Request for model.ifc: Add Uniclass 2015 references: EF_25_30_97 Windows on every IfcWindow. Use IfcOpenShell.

First a look at what the model holds.

```python
import ifcopenshell

model = ifcopenshell.open("model.ifc")
print(model.schema)
print("classifications:", [c.Name for c in model.by_type("IfcClassification")])
for ifc_class in ("IfcDoor", "IfcRoof", "IfcStair", "IfcWall", "IfcWindow"):
    print(ifc_class, len(model.by_type(ifc_class)))
```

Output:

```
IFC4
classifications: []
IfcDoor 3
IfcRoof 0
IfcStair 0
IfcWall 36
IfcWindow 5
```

```python
import ifcopenshell
import ifcopenshell.api.classification

model = ifcopenshell.open("model.ifc")

system = ifcopenshell.api.classification.add_classification(model, classification="Uniclass 2015")

codes = {
    "IfcWindow": ("EF_25_30_97", "Windows"),
}
for ifc_class, (code, name) in codes.items():
    products = model.by_type(ifc_class)
    ifcopenshell.api.classification.add_reference(
        model, products=products, classification=system, identification=code, name=name
    )
    print(code, len(products))

model.write("model-out.ifc")
```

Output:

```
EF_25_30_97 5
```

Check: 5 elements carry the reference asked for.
